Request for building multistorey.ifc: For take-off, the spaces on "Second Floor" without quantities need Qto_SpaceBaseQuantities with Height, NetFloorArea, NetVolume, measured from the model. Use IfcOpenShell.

First a look at what the model holds.

```python
import ifcopenshell
import ifcopenshell.util.element
import ifcopenshell.util.unit

model = ifcopenshell.open("building multistorey.ifc")
print(model.schema)
for unit_type in ("LENGTHUNIT", "AREAUNIT", "VOLUMEUNIT"):
    print(unit_type, ifcopenshell.util.unit.calculate_unit_scale(model, unit_type))
storey = next(s for s in model.by_type("IfcBuildingStorey") if s.Name == "Second Floor")
spaces = [e for e in ifcopenshell.util.element.get_decomposition(storey) if e.is_a("IfcSpace")]
for e in sorted(spaces, key=lambda e: e.id()):
    print(e.id(), e.is_a(), e.Name, list(ifcopenshell.util.element.get_psets(e, qtos_only=True)), sep=" | ")
```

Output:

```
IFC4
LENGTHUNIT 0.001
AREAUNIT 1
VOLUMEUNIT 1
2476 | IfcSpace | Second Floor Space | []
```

```python
import ifcopenshell
import ifcopenshell.api.pset
import ifcopenshell.geom
import ifcopenshell.util.element
import ifcopenshell.util.shape
import ifcopenshell.util.unit

model = ifcopenshell.open("building multistorey.ifc")
unit_scale = ifcopenshell.util.unit.calculate_unit_scale(model)
area_scale = ifcopenshell.util.unit.calculate_unit_scale(model, "AREAUNIT")
volume_scale = ifcopenshell.util.unit.calculate_unit_scale(model, "VOLUMEUNIT")
settings = ifcopenshell.geom.settings()

storey = next(s for s in model.by_type("IfcBuildingStorey") if s.Name == "Second Floor")
spaces = [e for e in ifcopenshell.util.element.get_decomposition(storey) if e.is_a("IfcSpace")]

for e in sorted(spaces, key=lambda e: e.id()):
    if ifcopenshell.util.element.get_psets(e, qtos_only=True, should_inherit=False):
        continue
    # Geometry comes back in metres, in the element's own axes.
    shape = ifcopenshell.geom.create_shape(settings, e)
    values = {
        "Height": ifcopenshell.util.shape.get_z(shape.geometry) / unit_scale,
        "NetFloorArea": ifcopenshell.util.shape.get_footprint_area(shape.geometry) / area_scale,
        "NetVolume": ifcopenshell.util.shape.get_volume(shape.geometry) / volume_scale,
    }
    qto = ifcopenshell.api.pset.add_qto(model, product=e, name="Qto_SpaceBaseQuantities")
    ifcopenshell.api.pset.edit_qto(model, qto=qto, properties=values)
    print(e.id(), {k: round(v, 3) for k, v in values.items()})

model.write("building multistorey_edited.ifc")
```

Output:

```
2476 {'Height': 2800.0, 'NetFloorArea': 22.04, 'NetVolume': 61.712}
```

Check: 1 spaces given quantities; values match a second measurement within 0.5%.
